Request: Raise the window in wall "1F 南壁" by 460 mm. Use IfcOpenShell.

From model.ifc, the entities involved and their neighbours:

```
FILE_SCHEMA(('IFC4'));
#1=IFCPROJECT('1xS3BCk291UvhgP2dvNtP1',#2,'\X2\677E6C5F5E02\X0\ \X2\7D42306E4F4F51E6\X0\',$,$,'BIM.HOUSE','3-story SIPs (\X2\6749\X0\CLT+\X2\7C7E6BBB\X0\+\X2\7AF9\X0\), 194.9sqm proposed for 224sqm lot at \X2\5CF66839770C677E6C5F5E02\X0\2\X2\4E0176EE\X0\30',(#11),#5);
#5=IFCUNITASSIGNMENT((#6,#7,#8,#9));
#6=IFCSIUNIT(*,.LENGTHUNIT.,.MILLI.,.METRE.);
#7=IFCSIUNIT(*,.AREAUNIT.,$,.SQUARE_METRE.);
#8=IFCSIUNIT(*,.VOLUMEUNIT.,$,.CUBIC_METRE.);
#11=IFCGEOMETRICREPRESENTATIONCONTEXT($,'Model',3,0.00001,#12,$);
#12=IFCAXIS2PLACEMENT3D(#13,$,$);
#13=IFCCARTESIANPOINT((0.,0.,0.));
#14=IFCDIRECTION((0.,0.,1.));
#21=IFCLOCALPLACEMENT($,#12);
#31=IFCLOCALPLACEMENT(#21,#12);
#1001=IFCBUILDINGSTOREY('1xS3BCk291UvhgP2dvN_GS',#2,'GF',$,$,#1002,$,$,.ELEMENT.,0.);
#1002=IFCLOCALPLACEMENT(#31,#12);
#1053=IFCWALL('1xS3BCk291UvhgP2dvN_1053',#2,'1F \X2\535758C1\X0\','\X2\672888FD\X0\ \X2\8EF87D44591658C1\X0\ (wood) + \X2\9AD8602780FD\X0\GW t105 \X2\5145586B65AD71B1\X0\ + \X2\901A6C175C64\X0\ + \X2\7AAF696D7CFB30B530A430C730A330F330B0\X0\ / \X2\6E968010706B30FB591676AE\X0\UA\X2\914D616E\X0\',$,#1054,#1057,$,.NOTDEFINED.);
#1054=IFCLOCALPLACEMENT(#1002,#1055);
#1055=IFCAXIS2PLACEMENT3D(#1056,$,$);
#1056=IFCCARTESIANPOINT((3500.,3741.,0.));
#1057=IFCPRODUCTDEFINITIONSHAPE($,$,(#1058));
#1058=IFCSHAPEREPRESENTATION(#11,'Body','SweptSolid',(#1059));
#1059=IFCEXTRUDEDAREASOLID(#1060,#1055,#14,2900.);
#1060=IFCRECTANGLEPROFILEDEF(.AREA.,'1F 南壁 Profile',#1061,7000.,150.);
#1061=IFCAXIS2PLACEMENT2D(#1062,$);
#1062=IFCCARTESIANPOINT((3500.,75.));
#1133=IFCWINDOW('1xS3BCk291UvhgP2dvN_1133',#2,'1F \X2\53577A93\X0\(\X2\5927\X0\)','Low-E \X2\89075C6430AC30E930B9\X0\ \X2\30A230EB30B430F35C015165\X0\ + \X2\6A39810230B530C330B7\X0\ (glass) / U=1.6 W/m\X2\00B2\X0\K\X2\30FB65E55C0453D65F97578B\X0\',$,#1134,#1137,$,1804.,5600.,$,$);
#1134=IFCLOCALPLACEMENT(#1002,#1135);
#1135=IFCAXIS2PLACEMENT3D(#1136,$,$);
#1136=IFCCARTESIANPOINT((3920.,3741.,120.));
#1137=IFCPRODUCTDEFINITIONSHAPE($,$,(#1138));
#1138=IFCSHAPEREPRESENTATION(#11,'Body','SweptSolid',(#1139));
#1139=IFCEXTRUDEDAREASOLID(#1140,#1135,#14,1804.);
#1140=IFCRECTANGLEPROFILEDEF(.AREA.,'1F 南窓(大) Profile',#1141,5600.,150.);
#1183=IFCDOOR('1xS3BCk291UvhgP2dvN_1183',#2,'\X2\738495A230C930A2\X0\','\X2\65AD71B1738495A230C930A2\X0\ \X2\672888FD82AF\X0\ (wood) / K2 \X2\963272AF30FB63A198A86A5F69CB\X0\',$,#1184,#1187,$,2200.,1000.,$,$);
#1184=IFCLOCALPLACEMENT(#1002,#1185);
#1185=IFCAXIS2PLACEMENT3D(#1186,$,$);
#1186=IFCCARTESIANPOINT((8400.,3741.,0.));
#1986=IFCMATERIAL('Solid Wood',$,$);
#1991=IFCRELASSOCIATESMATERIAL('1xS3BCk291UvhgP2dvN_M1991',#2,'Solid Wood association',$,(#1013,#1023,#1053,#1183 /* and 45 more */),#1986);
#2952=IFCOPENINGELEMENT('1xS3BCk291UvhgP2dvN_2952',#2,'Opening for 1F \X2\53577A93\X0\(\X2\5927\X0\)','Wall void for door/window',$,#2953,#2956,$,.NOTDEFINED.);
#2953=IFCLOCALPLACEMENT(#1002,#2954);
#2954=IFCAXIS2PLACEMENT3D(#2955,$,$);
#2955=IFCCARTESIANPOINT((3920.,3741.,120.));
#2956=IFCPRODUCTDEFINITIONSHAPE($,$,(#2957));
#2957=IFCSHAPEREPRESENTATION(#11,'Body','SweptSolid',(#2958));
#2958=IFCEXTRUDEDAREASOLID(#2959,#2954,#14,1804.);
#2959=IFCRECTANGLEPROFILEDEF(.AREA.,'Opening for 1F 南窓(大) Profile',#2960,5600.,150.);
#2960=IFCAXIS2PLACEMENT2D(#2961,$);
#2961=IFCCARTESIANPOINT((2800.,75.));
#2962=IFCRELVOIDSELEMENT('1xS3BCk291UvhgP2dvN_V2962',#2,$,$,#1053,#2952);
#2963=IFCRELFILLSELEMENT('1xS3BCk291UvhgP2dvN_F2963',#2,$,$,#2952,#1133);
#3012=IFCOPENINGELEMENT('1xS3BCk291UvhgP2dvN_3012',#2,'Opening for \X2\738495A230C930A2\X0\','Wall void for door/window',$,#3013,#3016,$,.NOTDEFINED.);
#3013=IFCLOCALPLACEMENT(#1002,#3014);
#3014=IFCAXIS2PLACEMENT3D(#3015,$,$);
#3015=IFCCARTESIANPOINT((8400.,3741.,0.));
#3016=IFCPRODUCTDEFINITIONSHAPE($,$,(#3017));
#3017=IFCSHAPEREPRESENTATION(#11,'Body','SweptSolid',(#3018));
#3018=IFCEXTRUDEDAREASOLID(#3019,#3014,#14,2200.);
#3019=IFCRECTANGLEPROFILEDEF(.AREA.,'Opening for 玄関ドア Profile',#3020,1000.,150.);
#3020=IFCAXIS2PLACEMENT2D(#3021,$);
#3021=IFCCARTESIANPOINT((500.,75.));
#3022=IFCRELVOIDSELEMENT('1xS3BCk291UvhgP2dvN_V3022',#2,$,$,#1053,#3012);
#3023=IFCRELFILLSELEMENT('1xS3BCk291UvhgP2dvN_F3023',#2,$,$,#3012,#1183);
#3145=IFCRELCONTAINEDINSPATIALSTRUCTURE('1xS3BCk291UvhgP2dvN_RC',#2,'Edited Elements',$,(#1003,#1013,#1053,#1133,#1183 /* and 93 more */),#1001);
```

```python
import numpy as np
import ifcopenshell
import ifcopenshell.api.geometry
import ifcopenshell.util.placement
import ifcopenshell.util.unit

model = ifcopenshell.open("model.ifc")
unit_scale = ifcopenshell.util.unit.calculate_unit_scale(model)

window = model.by_guid("1xS3BCk291UvhgP2dvN_1133")
opening = window.FillsVoids[0].RelatingOpeningElement
dz = 0.46 / unit_scale

shift = np.array([0.0, 0.0, dz])
# The window is not placed relative to its opening, so move both.
for product in (opening, window):
    matrix = ifcopenshell.util.placement.get_local_placement(product.ObjectPlacement)
    matrix[:3, 3] += shift
    ifcopenshell.api.geometry.edit_object_placement(model, product=product, matrix=matrix, is_si=False)

print(f"moved by {dz * unit_scale:+.3f} m")

model.write("model-out.ifc")
```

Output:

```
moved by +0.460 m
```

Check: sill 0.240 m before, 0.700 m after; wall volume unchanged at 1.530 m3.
